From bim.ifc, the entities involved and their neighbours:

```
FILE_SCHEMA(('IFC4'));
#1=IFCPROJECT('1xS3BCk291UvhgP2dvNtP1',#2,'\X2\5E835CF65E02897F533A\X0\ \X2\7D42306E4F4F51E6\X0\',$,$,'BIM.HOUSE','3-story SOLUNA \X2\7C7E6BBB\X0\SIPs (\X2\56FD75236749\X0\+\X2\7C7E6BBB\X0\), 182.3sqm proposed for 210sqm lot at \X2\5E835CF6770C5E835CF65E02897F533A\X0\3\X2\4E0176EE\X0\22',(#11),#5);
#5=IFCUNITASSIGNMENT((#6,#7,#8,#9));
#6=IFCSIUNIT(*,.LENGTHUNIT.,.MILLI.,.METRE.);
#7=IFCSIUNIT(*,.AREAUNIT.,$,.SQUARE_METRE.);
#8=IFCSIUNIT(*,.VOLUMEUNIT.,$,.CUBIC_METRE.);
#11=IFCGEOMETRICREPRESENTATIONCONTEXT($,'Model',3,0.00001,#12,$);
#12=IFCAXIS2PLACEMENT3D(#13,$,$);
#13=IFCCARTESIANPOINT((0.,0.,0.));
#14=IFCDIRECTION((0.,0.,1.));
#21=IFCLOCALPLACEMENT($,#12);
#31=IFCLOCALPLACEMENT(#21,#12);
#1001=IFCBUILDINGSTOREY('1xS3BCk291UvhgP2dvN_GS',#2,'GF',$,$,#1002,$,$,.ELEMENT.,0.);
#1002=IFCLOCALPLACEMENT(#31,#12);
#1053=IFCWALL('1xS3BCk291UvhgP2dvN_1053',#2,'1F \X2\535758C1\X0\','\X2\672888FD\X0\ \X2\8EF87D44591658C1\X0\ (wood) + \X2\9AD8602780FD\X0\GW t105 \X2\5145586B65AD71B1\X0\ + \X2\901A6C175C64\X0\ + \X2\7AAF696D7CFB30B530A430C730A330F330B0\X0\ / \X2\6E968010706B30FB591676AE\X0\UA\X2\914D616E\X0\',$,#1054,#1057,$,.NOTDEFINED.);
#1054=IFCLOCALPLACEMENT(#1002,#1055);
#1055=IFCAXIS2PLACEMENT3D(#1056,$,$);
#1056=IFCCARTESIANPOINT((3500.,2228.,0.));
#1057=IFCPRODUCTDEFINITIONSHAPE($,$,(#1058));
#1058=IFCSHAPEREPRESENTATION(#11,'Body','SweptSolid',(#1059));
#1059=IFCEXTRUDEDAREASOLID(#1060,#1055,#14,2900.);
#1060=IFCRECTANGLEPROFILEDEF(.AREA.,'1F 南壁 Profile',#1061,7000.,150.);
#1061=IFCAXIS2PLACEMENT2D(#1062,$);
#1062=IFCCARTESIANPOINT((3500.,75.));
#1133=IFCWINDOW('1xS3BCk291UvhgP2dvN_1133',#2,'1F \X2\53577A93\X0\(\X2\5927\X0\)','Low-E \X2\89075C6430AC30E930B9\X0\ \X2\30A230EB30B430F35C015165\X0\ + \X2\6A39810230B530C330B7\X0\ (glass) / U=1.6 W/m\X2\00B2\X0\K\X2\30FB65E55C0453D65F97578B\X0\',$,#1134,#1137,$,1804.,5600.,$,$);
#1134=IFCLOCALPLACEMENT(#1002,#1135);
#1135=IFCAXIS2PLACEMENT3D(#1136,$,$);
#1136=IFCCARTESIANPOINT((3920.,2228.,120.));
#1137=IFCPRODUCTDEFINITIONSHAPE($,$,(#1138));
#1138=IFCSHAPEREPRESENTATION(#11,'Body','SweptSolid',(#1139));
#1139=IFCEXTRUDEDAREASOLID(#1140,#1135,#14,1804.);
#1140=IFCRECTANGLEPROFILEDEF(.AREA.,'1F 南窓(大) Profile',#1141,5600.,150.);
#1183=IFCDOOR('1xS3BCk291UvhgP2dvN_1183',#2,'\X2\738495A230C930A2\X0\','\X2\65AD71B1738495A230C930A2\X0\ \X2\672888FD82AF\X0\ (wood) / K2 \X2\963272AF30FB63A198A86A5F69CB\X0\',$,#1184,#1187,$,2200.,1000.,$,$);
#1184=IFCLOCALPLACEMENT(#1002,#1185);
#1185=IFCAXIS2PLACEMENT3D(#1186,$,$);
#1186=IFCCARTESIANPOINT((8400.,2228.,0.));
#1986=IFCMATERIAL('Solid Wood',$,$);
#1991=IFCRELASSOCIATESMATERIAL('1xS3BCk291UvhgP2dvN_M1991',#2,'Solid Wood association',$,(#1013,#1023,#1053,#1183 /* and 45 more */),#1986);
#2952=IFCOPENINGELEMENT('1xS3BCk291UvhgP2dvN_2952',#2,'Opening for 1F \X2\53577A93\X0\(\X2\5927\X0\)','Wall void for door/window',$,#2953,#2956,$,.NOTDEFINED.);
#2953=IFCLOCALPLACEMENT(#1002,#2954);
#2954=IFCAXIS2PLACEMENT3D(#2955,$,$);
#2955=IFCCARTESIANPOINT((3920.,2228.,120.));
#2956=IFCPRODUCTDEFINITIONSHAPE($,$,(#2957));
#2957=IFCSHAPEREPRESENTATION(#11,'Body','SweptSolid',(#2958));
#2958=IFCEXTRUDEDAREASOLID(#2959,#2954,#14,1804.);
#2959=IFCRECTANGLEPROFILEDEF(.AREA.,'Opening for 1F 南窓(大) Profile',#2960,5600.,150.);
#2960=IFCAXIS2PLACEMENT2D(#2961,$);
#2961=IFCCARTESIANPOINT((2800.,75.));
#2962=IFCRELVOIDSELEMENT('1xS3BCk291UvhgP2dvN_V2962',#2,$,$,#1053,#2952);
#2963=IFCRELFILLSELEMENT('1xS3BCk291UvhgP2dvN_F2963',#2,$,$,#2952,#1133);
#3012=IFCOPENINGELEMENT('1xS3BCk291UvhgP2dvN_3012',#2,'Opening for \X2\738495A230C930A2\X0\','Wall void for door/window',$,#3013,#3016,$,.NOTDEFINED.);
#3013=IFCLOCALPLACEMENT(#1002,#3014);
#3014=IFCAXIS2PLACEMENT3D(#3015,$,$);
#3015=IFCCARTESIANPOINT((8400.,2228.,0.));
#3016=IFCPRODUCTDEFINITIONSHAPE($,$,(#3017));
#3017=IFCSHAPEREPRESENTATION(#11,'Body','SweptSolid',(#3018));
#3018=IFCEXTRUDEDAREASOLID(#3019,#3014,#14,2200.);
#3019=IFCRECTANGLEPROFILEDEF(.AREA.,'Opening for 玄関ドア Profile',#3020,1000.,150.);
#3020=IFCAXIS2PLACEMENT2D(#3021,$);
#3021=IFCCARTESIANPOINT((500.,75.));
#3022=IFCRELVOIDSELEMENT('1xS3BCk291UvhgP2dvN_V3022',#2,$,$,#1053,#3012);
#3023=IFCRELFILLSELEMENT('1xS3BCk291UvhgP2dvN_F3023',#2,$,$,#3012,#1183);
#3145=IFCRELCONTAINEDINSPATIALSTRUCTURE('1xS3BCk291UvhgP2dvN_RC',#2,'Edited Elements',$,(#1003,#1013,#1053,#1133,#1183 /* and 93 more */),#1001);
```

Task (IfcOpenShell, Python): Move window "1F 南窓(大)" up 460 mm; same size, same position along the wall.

```python
import numpy as np
import ifcopenshell
import ifcopenshell.api.geometry
import ifcopenshell.util.placement
import ifcopenshell.util.unit

model = ifcopenshell.open("bim.ifc")
unit_scale = ifcopenshell.util.unit.calculate_unit_scale(model)

window = model.by_guid("1xS3BCk291UvhgP2dvN_1133")
opening = window.FillsVoids[0].RelatingOpeningElement
dz = 460.0

shift = np.array([0.0, 0.0, dz])
# The window is not placed relative to its opening, so move both.
for product in (opening, window):
    matrix = ifcopenshell.util.placement.get_local_placement(product.ObjectPlacement)
    matrix[:3, 3] += shift
    ifcopenshell.api.geometry.edit_object_placement(model, product=product, matrix=matrix, is_si=False)

print(f"moved by {dz * unit_scale:+.3f} m")

model.write("bim-out.ifc")
```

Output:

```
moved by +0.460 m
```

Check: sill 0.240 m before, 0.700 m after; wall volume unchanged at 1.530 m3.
